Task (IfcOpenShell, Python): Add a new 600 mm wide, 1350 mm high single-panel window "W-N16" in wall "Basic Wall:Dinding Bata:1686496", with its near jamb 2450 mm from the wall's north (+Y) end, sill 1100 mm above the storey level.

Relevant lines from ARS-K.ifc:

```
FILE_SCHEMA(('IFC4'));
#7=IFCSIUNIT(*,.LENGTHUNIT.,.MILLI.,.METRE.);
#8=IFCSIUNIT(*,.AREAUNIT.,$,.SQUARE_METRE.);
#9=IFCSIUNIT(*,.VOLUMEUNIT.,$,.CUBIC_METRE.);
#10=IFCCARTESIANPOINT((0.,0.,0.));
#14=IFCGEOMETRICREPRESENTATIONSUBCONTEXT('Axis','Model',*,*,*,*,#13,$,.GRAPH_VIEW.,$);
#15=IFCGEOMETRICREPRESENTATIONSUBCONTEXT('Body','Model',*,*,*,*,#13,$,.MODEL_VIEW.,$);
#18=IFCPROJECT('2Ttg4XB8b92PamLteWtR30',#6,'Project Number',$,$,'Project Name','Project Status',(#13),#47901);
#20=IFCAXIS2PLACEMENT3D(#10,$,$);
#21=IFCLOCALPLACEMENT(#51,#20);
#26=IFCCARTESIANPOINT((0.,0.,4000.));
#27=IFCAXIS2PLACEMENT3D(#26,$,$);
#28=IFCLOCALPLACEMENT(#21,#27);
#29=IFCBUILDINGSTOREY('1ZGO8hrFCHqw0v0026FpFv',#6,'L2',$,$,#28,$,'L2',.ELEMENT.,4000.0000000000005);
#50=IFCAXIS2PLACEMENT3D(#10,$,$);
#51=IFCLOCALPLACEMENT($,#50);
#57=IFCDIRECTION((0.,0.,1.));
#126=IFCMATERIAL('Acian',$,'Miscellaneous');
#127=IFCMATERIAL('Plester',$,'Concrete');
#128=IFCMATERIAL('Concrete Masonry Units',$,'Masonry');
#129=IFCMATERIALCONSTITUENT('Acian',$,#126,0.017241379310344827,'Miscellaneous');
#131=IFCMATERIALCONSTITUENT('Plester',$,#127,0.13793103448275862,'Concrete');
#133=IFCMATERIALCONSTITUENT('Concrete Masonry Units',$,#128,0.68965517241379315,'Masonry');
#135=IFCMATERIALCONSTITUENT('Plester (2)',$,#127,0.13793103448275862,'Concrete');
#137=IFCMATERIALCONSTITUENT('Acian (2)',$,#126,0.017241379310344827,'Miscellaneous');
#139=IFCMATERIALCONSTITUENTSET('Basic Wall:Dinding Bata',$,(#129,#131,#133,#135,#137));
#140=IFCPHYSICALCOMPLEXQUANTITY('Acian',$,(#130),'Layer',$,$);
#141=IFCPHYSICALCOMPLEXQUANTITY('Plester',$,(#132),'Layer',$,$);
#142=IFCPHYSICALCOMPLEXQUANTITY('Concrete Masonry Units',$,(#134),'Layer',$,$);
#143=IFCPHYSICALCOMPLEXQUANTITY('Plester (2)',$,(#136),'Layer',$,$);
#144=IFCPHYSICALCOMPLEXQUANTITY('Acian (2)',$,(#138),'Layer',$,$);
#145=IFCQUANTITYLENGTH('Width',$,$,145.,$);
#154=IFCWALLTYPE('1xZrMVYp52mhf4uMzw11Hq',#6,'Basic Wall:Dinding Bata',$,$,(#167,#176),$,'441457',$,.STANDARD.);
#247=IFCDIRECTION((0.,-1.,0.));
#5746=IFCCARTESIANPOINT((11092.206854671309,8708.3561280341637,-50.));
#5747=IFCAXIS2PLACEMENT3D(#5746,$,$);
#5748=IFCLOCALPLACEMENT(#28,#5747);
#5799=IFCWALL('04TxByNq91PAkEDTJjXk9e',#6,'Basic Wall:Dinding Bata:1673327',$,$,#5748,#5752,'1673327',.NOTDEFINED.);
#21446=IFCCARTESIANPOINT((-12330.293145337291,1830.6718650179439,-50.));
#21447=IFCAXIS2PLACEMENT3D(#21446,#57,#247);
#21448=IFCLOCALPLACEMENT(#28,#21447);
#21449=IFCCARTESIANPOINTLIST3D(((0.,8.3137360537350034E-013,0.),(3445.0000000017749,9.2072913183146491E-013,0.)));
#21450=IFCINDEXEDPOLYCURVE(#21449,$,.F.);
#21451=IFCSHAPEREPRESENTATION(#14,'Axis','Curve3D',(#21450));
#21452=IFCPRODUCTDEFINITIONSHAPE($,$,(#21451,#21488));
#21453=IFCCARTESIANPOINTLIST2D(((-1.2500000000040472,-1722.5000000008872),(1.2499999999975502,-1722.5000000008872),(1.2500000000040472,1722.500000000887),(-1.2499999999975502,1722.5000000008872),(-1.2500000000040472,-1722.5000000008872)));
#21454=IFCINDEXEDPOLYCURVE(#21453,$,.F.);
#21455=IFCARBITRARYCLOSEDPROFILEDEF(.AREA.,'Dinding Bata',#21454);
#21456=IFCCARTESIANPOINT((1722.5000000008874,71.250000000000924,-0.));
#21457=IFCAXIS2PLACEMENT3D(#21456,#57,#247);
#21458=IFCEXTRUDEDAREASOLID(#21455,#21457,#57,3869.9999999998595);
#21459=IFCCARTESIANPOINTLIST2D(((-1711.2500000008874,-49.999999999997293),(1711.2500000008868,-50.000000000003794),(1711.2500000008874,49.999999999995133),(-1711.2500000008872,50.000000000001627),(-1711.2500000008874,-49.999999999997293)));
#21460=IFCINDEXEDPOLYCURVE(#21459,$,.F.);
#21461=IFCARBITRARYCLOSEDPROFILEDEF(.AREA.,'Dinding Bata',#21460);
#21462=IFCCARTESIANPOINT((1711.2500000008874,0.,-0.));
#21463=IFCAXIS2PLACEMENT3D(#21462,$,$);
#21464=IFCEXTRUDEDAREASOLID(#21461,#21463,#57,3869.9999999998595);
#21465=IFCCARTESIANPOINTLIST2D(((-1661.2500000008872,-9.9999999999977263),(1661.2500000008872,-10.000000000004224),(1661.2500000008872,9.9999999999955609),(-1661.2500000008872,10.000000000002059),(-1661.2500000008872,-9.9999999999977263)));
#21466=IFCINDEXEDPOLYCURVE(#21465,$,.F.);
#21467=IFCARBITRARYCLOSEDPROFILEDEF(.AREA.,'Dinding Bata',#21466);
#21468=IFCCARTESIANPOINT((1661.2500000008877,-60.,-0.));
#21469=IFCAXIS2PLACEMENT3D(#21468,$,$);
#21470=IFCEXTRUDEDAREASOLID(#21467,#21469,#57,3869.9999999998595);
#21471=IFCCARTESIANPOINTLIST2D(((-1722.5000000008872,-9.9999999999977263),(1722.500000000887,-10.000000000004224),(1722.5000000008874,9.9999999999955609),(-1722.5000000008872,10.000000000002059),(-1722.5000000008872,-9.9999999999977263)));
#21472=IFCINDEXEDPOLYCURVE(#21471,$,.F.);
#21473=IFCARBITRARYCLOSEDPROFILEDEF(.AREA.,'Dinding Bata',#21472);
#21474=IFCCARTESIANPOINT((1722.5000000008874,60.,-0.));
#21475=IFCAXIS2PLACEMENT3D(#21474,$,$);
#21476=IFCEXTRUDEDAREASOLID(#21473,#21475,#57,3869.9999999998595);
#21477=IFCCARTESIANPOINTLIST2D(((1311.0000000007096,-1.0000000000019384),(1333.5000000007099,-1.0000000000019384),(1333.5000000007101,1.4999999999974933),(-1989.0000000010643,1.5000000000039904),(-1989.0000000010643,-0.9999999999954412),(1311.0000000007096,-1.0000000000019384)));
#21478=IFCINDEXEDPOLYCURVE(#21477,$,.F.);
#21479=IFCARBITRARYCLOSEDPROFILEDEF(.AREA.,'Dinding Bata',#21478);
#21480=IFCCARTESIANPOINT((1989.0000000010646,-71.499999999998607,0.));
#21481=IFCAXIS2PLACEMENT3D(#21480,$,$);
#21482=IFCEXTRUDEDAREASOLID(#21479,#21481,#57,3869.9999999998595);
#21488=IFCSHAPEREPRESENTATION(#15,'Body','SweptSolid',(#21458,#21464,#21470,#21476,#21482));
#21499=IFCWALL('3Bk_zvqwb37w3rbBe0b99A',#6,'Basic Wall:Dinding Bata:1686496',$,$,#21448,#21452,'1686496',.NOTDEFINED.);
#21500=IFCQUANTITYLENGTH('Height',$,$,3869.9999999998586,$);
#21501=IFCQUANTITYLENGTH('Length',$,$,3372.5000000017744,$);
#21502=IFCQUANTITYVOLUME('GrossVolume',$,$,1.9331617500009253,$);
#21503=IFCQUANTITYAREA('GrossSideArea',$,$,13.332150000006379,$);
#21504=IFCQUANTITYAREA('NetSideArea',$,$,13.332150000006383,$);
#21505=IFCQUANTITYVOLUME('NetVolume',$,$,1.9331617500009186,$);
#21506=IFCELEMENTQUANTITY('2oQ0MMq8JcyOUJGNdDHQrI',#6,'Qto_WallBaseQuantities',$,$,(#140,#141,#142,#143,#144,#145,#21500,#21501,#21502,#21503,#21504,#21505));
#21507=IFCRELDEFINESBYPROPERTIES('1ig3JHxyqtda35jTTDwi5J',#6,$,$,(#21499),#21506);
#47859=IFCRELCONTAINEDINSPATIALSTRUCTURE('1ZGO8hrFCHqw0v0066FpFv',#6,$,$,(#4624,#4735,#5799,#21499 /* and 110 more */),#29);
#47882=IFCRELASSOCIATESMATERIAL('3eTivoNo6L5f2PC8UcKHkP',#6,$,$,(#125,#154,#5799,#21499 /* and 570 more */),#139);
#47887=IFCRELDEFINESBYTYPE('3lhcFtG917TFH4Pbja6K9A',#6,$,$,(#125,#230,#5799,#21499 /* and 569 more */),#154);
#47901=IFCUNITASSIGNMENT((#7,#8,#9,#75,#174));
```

```python
import numpy as np
import ifcopenshell
import ifcopenshell.api.feature
import ifcopenshell.api.geometry
import ifcopenshell.api.pset
import ifcopenshell.api.root
import ifcopenshell.api.spatial
import ifcopenshell.geom
import ifcopenshell.util.element
import ifcopenshell.util.placement
import ifcopenshell.util.representation
import ifcopenshell.util.shape
import ifcopenshell.util.unit

model = ifcopenshell.open("ARS-K.ifc")
unit_scale = ifcopenshell.util.unit.calculate_unit_scale(model)
area_scale = ifcopenshell.util.unit.calculate_unit_scale(model, "AREAUNIT")
volume_scale = ifcopenshell.util.unit.calculate_unit_scale(model, "VOLUMEUNIT")
settings = ifcopenshell.geom.settings()


def volume(element):
    """Net volume in cubic metres, openings subtracted."""
    shape = ifcopenshell.geom.create_shape(settings, element)
    return ifcopenshell.util.shape.get_volume(shape.geometry)


wall = model.by_guid("3Bk_zvqwb37w3rbBe0b99A")
storey = ifcopenshell.util.element.get_container(wall, ifc_class="IfcBuildingStorey")
context = ifcopenshell.util.representation.get_context(model, "Model", "Body", "MODEL_VIEW")
before = volume(wall)

width, height, from_end, sill = 0.6, 1.35, 2.45, 1.1  # metres

# The wall runs along its own X axis, and the end named is its -X end.
wall_shape = ifcopenshell.geom.create_shape(settings, wall)
x, y, z = ifcopenshell.util.shape.get_vertices(wall_shape.geometry).T
start = x.min() + from_end
face, thickness = float(y.min()), float(y.max() - y.min())
wall_matrix = ifcopenshell.util.placement.get_local_placement(wall.ObjectPlacement)
level = ifcopenshell.util.placement.get_local_placement(storey.ObjectPlacement)[2, 3]


def in_wall(x, y):
    """Placement at x, y metres in the wall's axes, at sill height."""
    matrix = wall_matrix.copy()
    matrix[:, 3] = wall_matrix @ np.array([x / unit_scale, y / unit_scale, 0.0, 1.0])
    matrix[2, 3] = level + sill / unit_scale
    return matrix


# Opening: a box that overshoots both wall faces by 50 mm.
opening = ifcopenshell.api.root.create_entity(model, ifc_class="IfcOpeningElement", predefined_type="OPENING")
box = ifcopenshell.api.geometry.add_wall_representation(
    model, context=context, length=width, height=height, thickness=thickness + 0.1
)
ifcopenshell.api.geometry.assign_representation(model, product=opening, representation=box)
ifcopenshell.api.geometry.edit_object_placement(model, product=opening, matrix=in_wall(start, face - 0.05), is_si=False)
ifcopenshell.api.feature.add_feature(model, feature=opening, element=wall)

window = ifcopenshell.api.root.create_entity(model, ifc_class="IfcWindow", name="W-N16", predefined_type="WINDOW")
window.OverallWidth, window.OverallHeight = width / unit_scale, height / unit_scale
window.PartitioningType = "SINGLE_PANEL"
body = ifcopenshell.api.geometry.add_window_representation(
    model,
    context=context,
    overall_width=window.OverallWidth,
    overall_height=window.OverallHeight,
    partition_type="SINGLE_PANEL",
)
ifcopenshell.api.geometry.assign_representation(model, product=window, representation=body)
ifcopenshell.api.spatial.assign_container(model, products=[window], relating_structure=storey)
ifcopenshell.api.feature.add_filling(model, opening=opening, element=window)

# Centre the window in the wall's thickness.
ifcopenshell.api.geometry.edit_object_placement(model, product=window, matrix=in_wall(start, face), is_si=False)
window_shape = ifcopenshell.geom.create_shape(settings, window)
depth = ifcopenshell.util.shape.get_vertices(window_shape.geometry)[:, 1]
offset = face + thickness / 2 - (depth.min() + depth.max()) / 2
ifcopenshell.api.geometry.edit_object_placement(model, product=window, matrix=in_wall(start, offset), is_si=False)

after = volume(wall)

# Update the wall's stored quantities.
qto = model.by_id(ifcopenshell.util.element.get_pset(wall, "Qto_WallBaseQuantities", should_inherit=False)["id"])
ifcopenshell.api.pset.edit_qto(model, qto=qto, properties={
    "NetSideArea": after / thickness / area_scale,
    "NetVolume": after / volume_scale,
})

print(f"wall volume {before:.3f} -> {after:.3f} m3")

model.write("ARS-K_rev.ifc")
```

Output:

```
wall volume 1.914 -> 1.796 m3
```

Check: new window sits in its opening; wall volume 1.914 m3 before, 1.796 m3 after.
